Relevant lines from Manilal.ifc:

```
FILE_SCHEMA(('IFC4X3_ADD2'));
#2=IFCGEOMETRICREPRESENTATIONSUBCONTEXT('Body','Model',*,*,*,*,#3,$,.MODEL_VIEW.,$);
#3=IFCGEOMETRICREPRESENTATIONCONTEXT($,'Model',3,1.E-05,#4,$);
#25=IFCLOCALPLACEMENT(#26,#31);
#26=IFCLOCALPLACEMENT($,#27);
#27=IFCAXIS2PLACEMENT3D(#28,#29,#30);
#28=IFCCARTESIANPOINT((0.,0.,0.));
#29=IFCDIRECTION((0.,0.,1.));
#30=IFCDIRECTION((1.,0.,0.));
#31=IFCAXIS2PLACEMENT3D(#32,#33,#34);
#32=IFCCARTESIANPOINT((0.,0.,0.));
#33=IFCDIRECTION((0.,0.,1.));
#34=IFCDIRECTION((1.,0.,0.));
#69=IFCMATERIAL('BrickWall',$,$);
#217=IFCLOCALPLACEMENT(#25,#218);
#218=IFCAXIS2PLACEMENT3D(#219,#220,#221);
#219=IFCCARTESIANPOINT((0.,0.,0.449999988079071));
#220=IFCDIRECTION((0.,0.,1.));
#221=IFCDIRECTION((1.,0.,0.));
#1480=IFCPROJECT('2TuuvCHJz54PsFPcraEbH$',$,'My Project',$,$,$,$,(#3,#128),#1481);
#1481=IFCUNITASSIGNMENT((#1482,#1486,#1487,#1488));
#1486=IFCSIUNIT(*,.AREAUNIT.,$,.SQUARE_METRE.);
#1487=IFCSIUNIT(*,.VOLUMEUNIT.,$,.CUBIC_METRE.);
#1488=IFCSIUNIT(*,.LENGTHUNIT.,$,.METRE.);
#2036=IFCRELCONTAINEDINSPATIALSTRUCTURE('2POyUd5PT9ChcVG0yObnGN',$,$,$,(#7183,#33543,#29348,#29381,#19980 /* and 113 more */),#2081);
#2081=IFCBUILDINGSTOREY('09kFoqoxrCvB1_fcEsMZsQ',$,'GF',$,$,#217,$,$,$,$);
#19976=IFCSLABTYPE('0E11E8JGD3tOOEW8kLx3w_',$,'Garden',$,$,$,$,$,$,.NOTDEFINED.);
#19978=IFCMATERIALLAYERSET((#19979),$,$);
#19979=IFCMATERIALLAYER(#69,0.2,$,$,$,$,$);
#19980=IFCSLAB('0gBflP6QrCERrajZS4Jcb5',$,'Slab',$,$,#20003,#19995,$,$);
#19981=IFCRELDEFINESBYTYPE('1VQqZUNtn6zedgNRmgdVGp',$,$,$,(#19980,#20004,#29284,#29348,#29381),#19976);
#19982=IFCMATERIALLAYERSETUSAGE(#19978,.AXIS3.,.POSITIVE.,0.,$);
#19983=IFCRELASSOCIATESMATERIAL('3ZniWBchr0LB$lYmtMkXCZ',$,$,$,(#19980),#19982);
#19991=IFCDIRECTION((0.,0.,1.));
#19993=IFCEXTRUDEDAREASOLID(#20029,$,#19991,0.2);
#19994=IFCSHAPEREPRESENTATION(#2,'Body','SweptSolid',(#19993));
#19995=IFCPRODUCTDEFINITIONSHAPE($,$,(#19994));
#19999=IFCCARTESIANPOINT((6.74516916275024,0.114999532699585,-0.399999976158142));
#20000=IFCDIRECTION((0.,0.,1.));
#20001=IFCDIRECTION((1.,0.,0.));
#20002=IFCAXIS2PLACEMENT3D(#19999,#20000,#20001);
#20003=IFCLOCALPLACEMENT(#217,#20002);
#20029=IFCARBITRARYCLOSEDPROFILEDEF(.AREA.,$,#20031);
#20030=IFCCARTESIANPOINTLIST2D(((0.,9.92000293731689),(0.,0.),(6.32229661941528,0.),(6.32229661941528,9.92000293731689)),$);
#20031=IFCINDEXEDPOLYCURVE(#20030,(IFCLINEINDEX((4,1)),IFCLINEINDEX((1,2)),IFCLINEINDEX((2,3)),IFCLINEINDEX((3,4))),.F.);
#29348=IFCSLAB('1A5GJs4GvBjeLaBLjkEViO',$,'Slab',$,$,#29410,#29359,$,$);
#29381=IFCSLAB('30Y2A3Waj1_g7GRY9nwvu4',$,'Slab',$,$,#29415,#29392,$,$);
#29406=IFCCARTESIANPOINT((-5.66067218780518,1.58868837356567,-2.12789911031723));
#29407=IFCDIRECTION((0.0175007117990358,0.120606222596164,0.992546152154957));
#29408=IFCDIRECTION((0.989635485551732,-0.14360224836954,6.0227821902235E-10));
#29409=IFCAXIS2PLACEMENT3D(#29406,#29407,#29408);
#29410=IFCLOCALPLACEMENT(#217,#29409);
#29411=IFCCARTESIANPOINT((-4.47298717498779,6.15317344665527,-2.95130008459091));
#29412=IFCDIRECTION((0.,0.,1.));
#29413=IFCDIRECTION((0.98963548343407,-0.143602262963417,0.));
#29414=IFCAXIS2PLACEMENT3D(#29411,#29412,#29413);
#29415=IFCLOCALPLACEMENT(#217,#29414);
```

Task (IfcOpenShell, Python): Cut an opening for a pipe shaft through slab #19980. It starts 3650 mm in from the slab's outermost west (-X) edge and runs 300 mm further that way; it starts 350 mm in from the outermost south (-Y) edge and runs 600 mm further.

```python
import numpy as np
import ifcopenshell
import ifcopenshell.api.feature
import ifcopenshell.api.geometry
import ifcopenshell.api.root
import ifcopenshell.geom
import ifcopenshell.util.placement
import ifcopenshell.util.representation
import ifcopenshell.util.shape
import ifcopenshell.util.unit

model = ifcopenshell.open("Manilal.ifc")
unit_scale = ifcopenshell.util.unit.calculate_unit_scale(model)
settings = ifcopenshell.geom.settings()


def volume(element):
    """Net volume in cubic metres, openings subtracted."""
    shape = ifcopenshell.geom.create_shape(settings, element)
    return ifcopenshell.util.shape.get_volume(shape.geometry)


slab = model.by_guid("0gBflP6QrCERrajZS4Jcb5")
before = volume(slab)

# Extent in the slab's own axes, in metres. The edges named are its -X and -Y sides.
slab_shape = ifcopenshell.geom.create_shape(settings, slab)
vertices = ifcopenshell.util.shape.get_vertices(slab_shape.geometry)
x_min, y_min, bottom = vertices.min(axis=0)
top = vertices[:, 2].max()

opening = ifcopenshell.api.root.create_entity(model, ifc_class="IfcOpeningElement", name="Pipe shaft opening", predefined_type="OPENING")
context = ifcopenshell.util.representation.get_context(model, "Model", "Body", "MODEL_VIEW")
width, depth = 0.3, 0.6
outline = [(0.0, 0.0), (width, 0.0), (width, depth), (0.0, depth), (0.0, 0.0)]
# Overshoot both faces by 50 mm so the cut is clean.
shape = ifcopenshell.api.geometry.add_slab_representation(
    model, context=context, depth=top - bottom + 0.1, polyline=outline
)
ifcopenshell.api.geometry.assign_representation(model, product=opening, representation=shape)

matrix = ifcopenshell.util.placement.get_local_placement(slab.ObjectPlacement)
matrix[:, 3] = matrix @ np.append(np.array([x_min + 3.65, y_min + 0.35, bottom - 0.05]) / unit_scale, 1.0)
ifcopenshell.api.geometry.edit_object_placement(model, product=opening, matrix=matrix, is_si=False)
ifcopenshell.api.feature.add_feature(model, feature=opening, element=slab)

after = volume(slab)

print(f"slab volume {before:.3f} -> {after:.3f} m3")

model.write("Manilal_v2.ifc")
```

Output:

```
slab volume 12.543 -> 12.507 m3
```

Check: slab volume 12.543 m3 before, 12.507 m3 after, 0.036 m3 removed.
